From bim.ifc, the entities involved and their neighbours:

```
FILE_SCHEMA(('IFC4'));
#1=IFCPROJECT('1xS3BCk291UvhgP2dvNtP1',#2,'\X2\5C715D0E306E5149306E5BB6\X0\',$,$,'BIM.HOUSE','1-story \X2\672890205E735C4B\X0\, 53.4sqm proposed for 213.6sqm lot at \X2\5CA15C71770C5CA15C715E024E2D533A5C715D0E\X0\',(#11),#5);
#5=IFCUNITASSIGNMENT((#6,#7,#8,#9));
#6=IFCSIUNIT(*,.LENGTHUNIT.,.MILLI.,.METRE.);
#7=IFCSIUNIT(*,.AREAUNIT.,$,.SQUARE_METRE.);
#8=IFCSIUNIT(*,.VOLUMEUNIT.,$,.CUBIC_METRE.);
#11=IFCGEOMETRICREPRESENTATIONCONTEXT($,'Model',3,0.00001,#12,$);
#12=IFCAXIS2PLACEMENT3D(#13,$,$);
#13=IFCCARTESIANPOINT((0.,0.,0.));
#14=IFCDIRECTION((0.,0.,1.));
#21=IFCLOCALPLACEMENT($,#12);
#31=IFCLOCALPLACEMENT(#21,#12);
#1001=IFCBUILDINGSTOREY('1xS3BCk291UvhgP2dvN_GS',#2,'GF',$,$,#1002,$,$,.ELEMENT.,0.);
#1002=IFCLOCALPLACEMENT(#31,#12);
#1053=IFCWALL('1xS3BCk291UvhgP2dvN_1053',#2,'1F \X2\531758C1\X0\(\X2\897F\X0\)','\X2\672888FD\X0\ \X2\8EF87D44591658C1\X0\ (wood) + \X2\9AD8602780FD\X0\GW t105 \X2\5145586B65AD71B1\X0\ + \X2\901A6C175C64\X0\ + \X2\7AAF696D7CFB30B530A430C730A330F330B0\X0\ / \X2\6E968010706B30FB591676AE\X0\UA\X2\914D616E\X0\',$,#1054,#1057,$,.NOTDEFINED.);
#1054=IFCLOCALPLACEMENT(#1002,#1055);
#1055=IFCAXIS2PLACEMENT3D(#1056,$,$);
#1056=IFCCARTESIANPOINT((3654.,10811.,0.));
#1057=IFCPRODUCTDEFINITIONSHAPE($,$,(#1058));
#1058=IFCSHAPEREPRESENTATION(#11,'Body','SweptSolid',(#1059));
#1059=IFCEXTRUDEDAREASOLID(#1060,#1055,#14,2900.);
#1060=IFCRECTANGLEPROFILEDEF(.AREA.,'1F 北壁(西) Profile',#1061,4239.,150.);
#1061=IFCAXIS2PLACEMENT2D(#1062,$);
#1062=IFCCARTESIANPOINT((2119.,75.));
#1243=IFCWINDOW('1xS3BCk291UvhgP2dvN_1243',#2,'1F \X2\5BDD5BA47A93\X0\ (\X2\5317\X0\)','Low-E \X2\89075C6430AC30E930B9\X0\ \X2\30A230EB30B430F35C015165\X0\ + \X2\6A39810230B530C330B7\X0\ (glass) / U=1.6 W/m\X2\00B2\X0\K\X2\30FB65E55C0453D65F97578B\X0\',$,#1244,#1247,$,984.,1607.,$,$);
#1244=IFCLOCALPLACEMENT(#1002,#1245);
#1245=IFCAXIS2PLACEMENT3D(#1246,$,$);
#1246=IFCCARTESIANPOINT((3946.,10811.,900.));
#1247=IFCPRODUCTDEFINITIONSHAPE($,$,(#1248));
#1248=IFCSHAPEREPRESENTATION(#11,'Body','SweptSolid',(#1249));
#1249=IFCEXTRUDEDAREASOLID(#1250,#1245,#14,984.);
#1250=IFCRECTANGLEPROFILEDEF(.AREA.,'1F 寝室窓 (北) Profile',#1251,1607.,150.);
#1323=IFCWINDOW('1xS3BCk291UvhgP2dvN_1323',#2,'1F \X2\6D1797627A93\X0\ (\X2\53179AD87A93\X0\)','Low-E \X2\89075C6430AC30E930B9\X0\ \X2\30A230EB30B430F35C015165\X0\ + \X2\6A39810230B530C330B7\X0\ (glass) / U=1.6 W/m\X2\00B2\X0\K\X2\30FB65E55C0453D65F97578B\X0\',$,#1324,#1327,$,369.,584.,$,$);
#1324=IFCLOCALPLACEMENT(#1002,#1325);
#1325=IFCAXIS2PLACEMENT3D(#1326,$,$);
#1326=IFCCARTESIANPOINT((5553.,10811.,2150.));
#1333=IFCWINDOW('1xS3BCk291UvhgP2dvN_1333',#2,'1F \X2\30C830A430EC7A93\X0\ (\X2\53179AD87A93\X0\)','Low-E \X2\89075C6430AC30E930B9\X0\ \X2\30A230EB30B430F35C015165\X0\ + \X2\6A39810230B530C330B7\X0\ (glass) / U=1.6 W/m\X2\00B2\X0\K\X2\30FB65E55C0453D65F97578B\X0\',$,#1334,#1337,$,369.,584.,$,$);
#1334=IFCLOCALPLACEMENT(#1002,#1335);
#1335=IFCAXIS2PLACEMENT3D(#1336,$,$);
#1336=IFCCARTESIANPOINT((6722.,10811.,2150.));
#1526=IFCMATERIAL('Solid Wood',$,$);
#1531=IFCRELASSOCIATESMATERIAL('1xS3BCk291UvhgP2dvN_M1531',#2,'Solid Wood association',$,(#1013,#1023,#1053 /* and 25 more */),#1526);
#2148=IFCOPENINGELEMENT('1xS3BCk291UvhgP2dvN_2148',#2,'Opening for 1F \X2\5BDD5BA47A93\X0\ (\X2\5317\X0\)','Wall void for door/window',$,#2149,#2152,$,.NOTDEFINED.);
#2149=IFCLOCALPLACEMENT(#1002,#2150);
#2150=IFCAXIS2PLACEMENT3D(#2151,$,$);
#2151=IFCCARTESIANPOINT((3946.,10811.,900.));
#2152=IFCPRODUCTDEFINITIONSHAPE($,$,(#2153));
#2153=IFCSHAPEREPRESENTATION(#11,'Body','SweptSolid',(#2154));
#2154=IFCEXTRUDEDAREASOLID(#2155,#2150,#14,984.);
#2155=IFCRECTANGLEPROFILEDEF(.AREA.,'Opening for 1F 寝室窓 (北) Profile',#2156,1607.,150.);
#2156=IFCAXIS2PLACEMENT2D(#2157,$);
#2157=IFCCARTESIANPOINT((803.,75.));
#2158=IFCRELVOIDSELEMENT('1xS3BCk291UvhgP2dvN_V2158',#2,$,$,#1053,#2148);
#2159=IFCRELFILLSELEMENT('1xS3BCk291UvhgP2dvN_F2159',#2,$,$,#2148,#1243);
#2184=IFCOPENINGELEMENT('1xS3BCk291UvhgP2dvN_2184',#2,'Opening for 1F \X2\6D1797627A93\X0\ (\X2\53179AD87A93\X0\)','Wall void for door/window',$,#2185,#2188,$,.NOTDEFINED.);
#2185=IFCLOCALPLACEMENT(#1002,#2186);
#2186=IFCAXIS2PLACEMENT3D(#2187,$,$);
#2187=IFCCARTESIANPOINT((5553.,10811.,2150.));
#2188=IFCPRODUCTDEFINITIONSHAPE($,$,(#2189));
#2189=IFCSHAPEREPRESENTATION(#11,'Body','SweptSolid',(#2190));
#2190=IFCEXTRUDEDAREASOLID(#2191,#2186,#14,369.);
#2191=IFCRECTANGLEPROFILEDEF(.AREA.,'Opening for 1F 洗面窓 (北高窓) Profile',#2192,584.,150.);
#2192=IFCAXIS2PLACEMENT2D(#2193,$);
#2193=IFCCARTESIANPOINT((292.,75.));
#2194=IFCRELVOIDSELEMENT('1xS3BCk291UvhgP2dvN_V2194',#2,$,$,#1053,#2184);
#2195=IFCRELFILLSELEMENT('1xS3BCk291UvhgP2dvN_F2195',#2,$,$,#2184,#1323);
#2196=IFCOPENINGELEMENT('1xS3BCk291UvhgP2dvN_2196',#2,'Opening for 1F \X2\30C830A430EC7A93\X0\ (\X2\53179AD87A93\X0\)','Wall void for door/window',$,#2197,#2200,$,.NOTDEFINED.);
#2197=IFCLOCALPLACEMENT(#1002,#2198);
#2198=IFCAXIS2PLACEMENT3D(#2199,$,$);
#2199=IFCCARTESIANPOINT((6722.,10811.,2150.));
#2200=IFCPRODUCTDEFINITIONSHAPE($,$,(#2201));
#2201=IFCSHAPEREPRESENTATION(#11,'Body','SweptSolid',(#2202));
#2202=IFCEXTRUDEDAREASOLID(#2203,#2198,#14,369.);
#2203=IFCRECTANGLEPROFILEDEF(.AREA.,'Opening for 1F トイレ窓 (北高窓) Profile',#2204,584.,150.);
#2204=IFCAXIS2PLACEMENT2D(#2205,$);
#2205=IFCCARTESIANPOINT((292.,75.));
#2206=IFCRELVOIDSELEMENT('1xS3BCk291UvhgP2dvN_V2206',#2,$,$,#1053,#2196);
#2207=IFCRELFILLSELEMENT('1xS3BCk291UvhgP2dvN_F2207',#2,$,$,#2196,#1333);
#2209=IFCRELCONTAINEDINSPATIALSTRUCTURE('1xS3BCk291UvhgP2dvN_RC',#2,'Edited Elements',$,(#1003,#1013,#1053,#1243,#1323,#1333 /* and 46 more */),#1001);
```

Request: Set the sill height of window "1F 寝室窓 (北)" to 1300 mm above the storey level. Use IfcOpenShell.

```python
import numpy as np
import ifcopenshell
import ifcopenshell.api.geometry
import ifcopenshell.geom
import ifcopenshell.util.element
import ifcopenshell.util.placement
import ifcopenshell.util.shape
import ifcopenshell.util.unit

model = ifcopenshell.open("bim.ifc")
unit_scale = ifcopenshell.util.unit.calculate_unit_scale(model)

window = model.by_guid("1xS3BCk291UvhgP2dvN_1243")
opening = window.FillsVoids[0].RelatingOpeningElement
storey = ifcopenshell.util.element.get_container(window, ifc_class="IfcBuildingStorey")
level = ifcopenshell.util.placement.get_local_placement(storey.ObjectPlacement)[2, 3]

# The opening's origin need not be at the sill, so measure its lowest point.
shape = ifcopenshell.geom.create_shape(ifcopenshell.geom.settings(), opening)
bottom = ifcopenshell.util.shape.get_shape_bottom_elevation(shape, shape.geometry) / unit_scale
dz = level + 1.3 / unit_scale - bottom

shift = np.array([0.0, 0.0, dz])
# The window is not placed relative to its opening, so move both.
for product in (opening, window):
    matrix = ifcopenshell.util.placement.get_local_placement(product.ObjectPlacement)
    matrix[:3, 3] += shift
    ifcopenshell.api.geometry.edit_object_placement(model, product=product, matrix=matrix, is_si=False)

print(f"moved by {dz * unit_scale:+.3f} m")

model.write("bim_edited.ifc")
```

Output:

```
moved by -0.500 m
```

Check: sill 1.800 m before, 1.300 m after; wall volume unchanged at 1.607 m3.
